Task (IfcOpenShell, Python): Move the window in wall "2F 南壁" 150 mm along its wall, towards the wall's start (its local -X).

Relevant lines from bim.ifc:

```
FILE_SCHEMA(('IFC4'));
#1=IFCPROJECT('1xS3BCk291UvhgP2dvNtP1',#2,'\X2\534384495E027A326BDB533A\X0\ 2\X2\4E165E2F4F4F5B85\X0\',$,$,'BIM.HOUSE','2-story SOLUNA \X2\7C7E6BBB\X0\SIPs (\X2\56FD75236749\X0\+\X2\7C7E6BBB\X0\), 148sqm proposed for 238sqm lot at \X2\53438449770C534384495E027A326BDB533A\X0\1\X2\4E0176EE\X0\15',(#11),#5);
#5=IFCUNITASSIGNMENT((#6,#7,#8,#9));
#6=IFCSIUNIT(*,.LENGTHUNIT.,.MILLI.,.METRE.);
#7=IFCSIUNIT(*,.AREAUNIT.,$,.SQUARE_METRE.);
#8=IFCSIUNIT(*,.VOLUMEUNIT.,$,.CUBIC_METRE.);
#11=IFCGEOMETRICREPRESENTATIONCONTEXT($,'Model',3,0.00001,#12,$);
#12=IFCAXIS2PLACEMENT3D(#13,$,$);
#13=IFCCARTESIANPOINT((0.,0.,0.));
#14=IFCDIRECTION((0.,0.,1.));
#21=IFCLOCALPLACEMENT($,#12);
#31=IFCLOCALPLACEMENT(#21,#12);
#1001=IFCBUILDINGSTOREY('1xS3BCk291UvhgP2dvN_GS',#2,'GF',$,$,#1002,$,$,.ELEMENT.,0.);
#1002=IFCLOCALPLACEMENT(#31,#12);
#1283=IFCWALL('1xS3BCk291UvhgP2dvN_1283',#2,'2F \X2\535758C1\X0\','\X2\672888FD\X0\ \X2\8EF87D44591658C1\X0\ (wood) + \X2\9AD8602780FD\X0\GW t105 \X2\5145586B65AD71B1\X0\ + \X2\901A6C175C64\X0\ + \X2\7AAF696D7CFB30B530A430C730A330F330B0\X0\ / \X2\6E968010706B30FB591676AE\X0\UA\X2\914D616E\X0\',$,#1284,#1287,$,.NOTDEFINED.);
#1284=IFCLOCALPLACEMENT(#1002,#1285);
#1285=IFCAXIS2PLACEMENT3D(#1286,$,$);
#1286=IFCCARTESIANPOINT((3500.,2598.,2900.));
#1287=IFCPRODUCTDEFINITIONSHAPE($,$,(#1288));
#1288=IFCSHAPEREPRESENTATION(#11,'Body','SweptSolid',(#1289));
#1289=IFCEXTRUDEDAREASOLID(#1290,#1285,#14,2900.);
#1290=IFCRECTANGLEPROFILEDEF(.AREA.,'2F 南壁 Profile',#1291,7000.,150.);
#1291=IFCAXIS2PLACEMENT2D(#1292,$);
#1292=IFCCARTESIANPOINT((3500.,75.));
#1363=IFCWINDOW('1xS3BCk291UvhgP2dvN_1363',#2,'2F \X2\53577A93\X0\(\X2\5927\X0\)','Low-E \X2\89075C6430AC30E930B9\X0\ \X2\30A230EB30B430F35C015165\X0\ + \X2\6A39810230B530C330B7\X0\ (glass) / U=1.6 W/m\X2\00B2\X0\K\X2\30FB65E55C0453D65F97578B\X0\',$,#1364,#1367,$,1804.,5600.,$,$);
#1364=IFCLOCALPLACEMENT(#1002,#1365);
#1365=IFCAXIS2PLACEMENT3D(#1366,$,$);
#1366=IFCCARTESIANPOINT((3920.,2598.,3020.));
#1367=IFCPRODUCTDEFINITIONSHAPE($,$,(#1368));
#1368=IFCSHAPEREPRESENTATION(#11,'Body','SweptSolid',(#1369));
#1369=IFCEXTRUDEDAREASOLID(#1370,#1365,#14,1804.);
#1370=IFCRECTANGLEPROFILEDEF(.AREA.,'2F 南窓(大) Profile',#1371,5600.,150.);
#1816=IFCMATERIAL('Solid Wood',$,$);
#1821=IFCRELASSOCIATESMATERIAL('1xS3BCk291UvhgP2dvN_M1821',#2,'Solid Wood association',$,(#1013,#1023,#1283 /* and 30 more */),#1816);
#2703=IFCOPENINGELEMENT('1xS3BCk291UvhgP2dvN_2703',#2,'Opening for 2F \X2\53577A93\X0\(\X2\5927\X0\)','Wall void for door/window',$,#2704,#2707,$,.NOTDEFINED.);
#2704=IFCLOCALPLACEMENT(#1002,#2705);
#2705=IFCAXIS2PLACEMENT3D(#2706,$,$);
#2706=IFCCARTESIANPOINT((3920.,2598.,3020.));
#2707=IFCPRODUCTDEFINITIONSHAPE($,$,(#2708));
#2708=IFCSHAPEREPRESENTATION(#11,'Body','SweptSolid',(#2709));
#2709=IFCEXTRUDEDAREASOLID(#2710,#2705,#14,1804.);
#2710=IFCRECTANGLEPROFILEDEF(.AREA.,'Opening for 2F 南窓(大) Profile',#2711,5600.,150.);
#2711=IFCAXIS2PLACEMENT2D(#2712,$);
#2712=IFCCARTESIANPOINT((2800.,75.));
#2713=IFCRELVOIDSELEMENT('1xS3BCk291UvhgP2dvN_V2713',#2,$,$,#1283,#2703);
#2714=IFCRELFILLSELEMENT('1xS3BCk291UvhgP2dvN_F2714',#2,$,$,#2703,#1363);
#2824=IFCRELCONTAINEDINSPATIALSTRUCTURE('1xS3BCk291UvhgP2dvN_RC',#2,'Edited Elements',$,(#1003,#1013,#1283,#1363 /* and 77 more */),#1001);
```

```python
import ifcopenshell
import ifcopenshell.api.geometry
import ifcopenshell.util.placement
import ifcopenshell.util.unit

model = ifcopenshell.open("bim.ifc")
unit_scale = ifcopenshell.util.unit.calculate_unit_scale(model)

window = model.by_guid("1xS3BCk291UvhgP2dvN_1363")
opening = window.FillsVoids[0].RelatingOpeningElement
wall = opening.VoidsElements[0].RelatingBuildingElement

wall_matrix = ifcopenshell.util.placement.get_local_placement(wall.ObjectPlacement)
shift = wall_matrix[:3, 0] * -0.15 / unit_scale
before = ifcopenshell.util.placement.get_local_placement(window.ObjectPlacement)[:3, 3].copy()

# The window is not placed relative to its opening, so move both.
for product in (opening, window):
    matrix = ifcopenshell.util.placement.get_local_placement(product.ObjectPlacement)
    matrix[:3, 3] += shift
    ifcopenshell.api.geometry.edit_object_placement(model, product=product, matrix=matrix, is_si=False)

after = ifcopenshell.util.placement.get_local_placement(window.ObjectPlacement)[:3, 3]
print("window moved by", (after - before).round(3) + 0.0)

model.write("bim_rev.ifc")
```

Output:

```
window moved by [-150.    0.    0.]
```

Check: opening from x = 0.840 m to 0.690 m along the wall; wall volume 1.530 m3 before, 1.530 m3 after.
